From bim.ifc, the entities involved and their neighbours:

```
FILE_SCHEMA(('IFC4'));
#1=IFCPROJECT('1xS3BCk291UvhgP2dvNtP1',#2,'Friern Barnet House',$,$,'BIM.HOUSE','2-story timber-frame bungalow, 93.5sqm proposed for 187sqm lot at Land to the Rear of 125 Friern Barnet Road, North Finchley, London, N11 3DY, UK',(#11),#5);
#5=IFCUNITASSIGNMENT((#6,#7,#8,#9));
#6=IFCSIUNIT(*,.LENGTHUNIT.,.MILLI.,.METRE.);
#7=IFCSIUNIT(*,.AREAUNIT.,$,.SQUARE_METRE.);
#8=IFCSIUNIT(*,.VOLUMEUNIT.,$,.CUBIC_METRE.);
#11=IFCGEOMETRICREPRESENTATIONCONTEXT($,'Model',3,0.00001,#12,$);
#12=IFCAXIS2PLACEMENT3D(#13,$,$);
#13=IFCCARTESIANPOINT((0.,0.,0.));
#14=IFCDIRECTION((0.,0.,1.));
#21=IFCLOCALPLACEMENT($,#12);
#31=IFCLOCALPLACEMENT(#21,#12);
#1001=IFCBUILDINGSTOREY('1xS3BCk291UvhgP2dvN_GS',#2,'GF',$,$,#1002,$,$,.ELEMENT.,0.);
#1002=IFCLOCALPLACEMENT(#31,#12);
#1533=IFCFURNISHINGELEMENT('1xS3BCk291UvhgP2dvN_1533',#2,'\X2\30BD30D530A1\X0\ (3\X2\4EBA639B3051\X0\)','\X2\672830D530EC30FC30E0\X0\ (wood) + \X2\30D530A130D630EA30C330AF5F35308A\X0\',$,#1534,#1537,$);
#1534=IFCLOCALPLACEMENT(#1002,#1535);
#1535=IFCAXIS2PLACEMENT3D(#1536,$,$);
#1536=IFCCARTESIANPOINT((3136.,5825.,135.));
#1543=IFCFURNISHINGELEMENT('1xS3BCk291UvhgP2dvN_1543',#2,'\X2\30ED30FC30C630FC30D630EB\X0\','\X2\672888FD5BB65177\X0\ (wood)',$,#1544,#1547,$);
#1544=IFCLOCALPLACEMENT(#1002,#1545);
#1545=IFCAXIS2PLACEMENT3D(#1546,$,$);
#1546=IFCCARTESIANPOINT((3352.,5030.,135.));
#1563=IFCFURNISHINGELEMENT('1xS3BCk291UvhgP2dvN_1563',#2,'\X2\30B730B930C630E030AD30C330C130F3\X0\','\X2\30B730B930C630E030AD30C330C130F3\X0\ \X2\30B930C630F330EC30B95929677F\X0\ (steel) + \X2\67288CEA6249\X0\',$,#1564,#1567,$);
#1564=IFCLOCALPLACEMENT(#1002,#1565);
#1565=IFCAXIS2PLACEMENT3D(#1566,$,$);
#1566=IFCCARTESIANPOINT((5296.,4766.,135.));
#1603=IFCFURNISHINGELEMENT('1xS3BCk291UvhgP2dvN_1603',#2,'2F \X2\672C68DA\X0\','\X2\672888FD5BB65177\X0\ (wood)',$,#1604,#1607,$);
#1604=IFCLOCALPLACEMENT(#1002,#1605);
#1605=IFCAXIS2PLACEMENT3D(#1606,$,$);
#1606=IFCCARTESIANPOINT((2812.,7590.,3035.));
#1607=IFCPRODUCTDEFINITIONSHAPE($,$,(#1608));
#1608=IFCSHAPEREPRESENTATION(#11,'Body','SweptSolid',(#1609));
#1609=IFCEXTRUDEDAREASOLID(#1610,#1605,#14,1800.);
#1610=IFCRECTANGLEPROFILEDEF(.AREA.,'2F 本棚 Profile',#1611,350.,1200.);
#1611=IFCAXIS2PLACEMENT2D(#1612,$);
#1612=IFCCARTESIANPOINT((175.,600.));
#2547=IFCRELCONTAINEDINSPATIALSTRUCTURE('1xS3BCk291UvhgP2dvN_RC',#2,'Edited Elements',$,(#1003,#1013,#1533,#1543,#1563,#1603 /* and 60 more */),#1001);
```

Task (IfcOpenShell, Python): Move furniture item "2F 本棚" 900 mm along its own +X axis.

```python
import ifcopenshell
import ifcopenshell.api.geometry
import ifcopenshell.util.placement
import ifcopenshell.util.unit

model = ifcopenshell.open("bim.ifc")
unit_scale = ifcopenshell.util.unit.calculate_unit_scale(model)

item = model.by_guid("1xS3BCk291UvhgP2dvN_1603")
matrix = ifcopenshell.util.placement.get_local_placement(item.ObjectPlacement)
matrix[:3, 3] += matrix[:3, 0] * 0.9 / unit_scale
ifcopenshell.api.geometry.edit_object_placement(model, product=item, matrix=matrix, is_si=False)

print(ifcopenshell.util.placement.get_local_placement(item.ObjectPlacement).round(3) + 0.0)

model.write("bim_v2.ifc")
```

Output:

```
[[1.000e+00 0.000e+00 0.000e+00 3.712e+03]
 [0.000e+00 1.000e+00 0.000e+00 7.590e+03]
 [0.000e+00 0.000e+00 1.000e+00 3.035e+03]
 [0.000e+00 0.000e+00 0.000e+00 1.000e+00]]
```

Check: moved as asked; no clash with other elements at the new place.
